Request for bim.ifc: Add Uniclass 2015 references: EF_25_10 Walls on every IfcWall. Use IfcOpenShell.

First a look at what the model holds.

```python
import ifcopenshell

model = ifcopenshell.open("bim.ifc")
print(model.schema)
print("classifications:", [c.Name for c in model.by_type("IfcClassification")])
for ifc_class in ("IfcDoor", "IfcRoof", "IfcStair", "IfcWall", "IfcWindow"):
    print(ifc_class, len(model.by_type(ifc_class)))
```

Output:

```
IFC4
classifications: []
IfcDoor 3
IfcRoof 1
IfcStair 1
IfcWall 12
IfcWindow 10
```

```python
import ifcopenshell
import ifcopenshell.api.classification

model = ifcopenshell.open("bim.ifc")

system = ifcopenshell.api.classification.add_classification(model, classification="Uniclass 2015")

codes = {
    "IfcWall": ("EF_25_10", "Walls"),
}
for ifc_class, (code, name) in codes.items():
    products = model.by_type(ifc_class)
    ifcopenshell.api.classification.add_reference(
        model, products=products, classification=system, identification=code, name=name
    )
    print(code, len(products))

model.write("bim_edited.ifc")
```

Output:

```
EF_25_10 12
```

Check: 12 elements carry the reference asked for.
